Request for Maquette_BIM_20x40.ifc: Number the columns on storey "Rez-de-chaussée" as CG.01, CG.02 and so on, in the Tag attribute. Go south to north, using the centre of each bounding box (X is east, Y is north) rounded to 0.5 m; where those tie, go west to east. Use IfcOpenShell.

First a look at what the model holds.

```python
import ifcopenshell
import ifcopenshell.util.element
import ifcopenshell.util.placement

model = ifcopenshell.open("Maquette_BIM_20x40.ifc")
print(model.schema)
storey = next(s for s in model.by_type("IfcBuildingStorey") if s.Name == "Rez-de-chaussée")
columns = [e for e in ifcopenshell.util.element.get_decomposition(storey) if e.is_a("IfcColumn")]
for e in sorted(columns, key=lambda e: e.id()):
    origin = ifcopenshell.util.placement.get_local_placement(e.ObjectPlacement)[:3, 3]
    print(e.id(), e.Tag, e.Name, origin.round(2) + 0.0, sep=" | ")
```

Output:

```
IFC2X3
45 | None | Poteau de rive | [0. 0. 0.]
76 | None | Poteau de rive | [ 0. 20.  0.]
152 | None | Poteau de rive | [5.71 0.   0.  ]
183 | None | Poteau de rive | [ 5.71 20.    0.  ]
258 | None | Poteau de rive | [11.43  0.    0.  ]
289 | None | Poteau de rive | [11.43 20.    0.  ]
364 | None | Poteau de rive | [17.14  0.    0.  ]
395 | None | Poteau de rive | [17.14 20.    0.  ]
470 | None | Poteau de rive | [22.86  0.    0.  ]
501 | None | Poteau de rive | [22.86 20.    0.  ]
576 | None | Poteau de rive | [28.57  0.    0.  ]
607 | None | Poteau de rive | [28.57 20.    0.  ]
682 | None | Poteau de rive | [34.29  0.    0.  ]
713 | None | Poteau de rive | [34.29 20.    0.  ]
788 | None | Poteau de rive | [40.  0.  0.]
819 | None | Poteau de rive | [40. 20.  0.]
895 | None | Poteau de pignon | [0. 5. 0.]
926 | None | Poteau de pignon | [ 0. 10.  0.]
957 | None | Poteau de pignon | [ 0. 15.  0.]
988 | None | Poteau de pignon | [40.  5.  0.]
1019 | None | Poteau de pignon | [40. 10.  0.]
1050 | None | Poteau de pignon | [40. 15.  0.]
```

```python
import ifcopenshell
import ifcopenshell.geom
import ifcopenshell.util.element
import ifcopenshell.util.shape

model = ifcopenshell.open("Maquette_BIM_20x40.ifc")
settings = ifcopenshell.geom.settings()
settings.set("use-world-coords", True)


def centre(element):
    shape = ifcopenshell.geom.create_shape(settings, element)
    return ifcopenshell.util.shape.get_bbox_centroid(shape.geometry)


storey = next(s for s in model.by_type("IfcBuildingStorey") if s.Name == "Rez-de-chaussée")
columns = [e for e in ifcopenshell.util.element.get_decomposition(storey) if e.is_a("IfcColumn")]

# Insertion points can sit at a corner or the storey origin, so sort by the geometry (in metres).
centres = {e: centre(e) for e in columns}
columns.sort(key=lambda e: (round(centres[e][1] / 0.5), centres[e][0]))

for i, e in enumerate(columns, start=1):
    number = f"CG.{i:02d}"
    e.Tag = number
    print(e.id(), number)

model.write("Maquette_BIM_20x40_edited.ifc")
```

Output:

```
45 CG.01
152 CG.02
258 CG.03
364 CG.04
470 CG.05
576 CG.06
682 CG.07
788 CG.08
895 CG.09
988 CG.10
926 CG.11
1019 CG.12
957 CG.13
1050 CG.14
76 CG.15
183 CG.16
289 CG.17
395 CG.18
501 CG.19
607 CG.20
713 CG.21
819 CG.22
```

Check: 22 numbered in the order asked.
